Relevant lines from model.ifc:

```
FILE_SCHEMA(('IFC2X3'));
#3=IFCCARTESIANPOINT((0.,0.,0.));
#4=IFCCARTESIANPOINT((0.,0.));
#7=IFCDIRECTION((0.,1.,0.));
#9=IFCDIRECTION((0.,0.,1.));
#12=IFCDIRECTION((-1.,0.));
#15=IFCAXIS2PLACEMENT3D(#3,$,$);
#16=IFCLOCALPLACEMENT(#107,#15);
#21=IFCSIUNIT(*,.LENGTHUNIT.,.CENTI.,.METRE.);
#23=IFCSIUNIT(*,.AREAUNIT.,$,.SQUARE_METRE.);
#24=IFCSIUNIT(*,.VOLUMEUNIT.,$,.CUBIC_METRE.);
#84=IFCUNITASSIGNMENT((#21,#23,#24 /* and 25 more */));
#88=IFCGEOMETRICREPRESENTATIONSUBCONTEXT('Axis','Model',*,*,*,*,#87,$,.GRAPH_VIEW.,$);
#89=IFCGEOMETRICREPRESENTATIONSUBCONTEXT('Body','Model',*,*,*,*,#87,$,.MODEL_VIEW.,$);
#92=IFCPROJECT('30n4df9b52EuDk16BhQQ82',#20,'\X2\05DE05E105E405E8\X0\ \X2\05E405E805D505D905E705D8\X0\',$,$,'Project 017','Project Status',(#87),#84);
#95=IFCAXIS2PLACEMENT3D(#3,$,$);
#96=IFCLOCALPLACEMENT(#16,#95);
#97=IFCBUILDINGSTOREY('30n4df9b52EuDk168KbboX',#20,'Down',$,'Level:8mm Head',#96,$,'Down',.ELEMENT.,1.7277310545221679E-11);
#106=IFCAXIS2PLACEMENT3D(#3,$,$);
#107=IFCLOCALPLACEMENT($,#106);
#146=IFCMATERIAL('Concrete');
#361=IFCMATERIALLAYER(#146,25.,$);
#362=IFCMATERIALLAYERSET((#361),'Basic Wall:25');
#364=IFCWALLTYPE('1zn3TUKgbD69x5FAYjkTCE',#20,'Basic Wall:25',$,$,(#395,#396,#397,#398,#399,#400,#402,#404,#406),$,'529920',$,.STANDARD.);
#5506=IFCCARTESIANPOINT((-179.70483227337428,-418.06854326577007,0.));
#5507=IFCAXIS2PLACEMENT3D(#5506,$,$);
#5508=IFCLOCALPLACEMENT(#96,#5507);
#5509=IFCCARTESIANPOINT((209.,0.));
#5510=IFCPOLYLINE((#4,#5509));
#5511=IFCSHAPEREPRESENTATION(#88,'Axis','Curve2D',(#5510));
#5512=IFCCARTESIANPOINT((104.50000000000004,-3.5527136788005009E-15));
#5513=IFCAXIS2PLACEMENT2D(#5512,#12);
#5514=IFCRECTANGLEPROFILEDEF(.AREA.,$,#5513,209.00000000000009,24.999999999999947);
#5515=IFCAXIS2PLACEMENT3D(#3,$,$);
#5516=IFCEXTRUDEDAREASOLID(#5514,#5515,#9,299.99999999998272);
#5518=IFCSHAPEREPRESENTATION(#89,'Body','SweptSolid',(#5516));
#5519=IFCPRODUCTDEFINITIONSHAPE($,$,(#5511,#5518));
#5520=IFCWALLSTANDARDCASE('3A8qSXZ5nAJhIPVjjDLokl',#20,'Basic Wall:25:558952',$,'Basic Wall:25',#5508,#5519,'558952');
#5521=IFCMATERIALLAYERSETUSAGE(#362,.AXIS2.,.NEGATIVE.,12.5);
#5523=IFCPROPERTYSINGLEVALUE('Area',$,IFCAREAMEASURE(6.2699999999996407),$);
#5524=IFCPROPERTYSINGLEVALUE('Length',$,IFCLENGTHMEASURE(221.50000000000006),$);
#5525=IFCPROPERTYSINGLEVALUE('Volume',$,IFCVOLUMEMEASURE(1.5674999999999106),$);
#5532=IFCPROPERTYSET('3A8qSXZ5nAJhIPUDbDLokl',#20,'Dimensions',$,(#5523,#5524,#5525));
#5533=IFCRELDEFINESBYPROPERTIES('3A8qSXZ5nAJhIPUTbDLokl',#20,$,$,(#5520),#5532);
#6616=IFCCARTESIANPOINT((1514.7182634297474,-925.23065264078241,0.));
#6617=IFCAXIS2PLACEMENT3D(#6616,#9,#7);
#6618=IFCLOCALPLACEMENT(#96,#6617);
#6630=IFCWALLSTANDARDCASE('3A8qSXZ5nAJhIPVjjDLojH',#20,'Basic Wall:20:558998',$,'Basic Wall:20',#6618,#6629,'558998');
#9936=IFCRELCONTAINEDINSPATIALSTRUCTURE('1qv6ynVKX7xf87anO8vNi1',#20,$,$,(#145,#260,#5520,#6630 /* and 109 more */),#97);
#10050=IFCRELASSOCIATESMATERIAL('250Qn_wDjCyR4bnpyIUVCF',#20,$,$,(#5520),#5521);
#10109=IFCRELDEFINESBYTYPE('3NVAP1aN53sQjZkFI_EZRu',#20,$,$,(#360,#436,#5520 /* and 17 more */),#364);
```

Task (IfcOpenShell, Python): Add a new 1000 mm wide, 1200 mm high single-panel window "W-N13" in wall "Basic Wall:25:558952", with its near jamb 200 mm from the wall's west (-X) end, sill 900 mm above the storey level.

```python
import numpy as np
import ifcopenshell
import ifcopenshell.api.feature
import ifcopenshell.api.geometry
import ifcopenshell.api.pset
import ifcopenshell.api.root
import ifcopenshell.api.spatial
import ifcopenshell.api.type
import ifcopenshell.geom
import ifcopenshell.util.element
import ifcopenshell.util.placement
import ifcopenshell.util.representation
import ifcopenshell.util.shape
import ifcopenshell.util.unit

model = ifcopenshell.open("model.ifc")
unit_scale = ifcopenshell.util.unit.calculate_unit_scale(model)
area_scale = ifcopenshell.util.unit.calculate_unit_scale(model, "AREAUNIT")
volume_scale = ifcopenshell.util.unit.calculate_unit_scale(model, "VOLUMEUNIT")
settings = ifcopenshell.geom.settings()


def volume(element):
    """Net volume in cubic metres, openings subtracted."""
    shape = ifcopenshell.geom.create_shape(settings, element)
    return ifcopenshell.util.shape.get_volume(shape.geometry)


wall = model.by_guid("3A8qSXZ5nAJhIPVjjDLokl")
storey = ifcopenshell.util.element.get_container(wall, ifc_class="IfcBuildingStorey")
context = ifcopenshell.util.representation.get_context(model, "Model", "Body", "MODEL_VIEW")
before = volume(wall)

width, height, from_end, sill = 1, 1.2, 0.2, 0.9  # metres

# The wall runs along its own X axis, and the end named is its -X end.
wall_shape = ifcopenshell.geom.create_shape(settings, wall)
x, y, z = ifcopenshell.util.shape.get_vertices(wall_shape.geometry).T
start = x.min() + from_end
face, thickness = float(y.min()), float(y.max() - y.min())
wall_matrix = ifcopenshell.util.placement.get_local_placement(wall.ObjectPlacement)
level = ifcopenshell.util.placement.get_local_placement(storey.ObjectPlacement)[2, 3]


def in_wall(x, y):
    """Placement at x, y metres in the wall's axes, at sill height."""
    matrix = wall_matrix.copy()
    matrix[:, 3] = wall_matrix @ np.array([x / unit_scale, y / unit_scale, 0.0, 1.0])
    matrix[2, 3] = level + sill / unit_scale
    return matrix


# Opening: a box that overshoots both wall faces by 50 mm.
opening = ifcopenshell.api.root.create_entity(model, ifc_class="IfcOpeningElement")
box = ifcopenshell.api.geometry.add_wall_representation(
    model, context=context, length=width, height=height, thickness=thickness + 0.1
)
ifcopenshell.api.geometry.assign_representation(model, product=opening, representation=box)
ifcopenshell.api.geometry.edit_object_placement(model, product=opening, matrix=in_wall(start, face - 0.05), is_si=False)
ifcopenshell.api.feature.add_feature(model, feature=opening, element=wall)

window = ifcopenshell.api.root.create_entity(model, ifc_class="IfcWindow", name="W-N13")
window.OverallWidth, window.OverallHeight = width / unit_scale, height / unit_scale
body = ifcopenshell.api.geometry.add_window_representation(
    model,
    context=context,
    overall_width=window.OverallWidth,
    overall_height=window.OverallHeight,
    partition_type="SINGLE_PANEL",
)
ifcopenshell.api.geometry.assign_representation(model, product=window, representation=body)
ifcopenshell.api.spatial.assign_container(model, products=[window], relating_structure=storey)
fills = ifcopenshell.api.feature.add_filling(model, opening=opening, element=window)
fills.OwnerHistory = window.OwnerHistory  # required in IFC2X3

# IFC2X3 keeps the operation on the window style.
style = ifcopenshell.api.root.create_entity(model, ifc_class="IfcWindowStyle", name="W-N13")
style.OperationType, style.ConstructionType = "SINGLE_PANEL", "NOTDEFINED"
style.ParameterTakesPrecedence = style.Sizeable = False
ifcopenshell.api.type.assign_type(model, related_objects=[window], relating_type=style)

# Centre the window in the wall's thickness.
ifcopenshell.api.geometry.edit_object_placement(model, product=window, matrix=in_wall(start, face), is_si=False)
window_shape = ifcopenshell.geom.create_shape(settings, window)
depth = ifcopenshell.util.shape.get_vertices(window_shape.geometry)[:, 1]
offset = face + thickness / 2 - (depth.min() + depth.max()) / 2
ifcopenshell.api.geometry.edit_object_placement(model, product=window, matrix=in_wall(start, offset), is_si=False)

after = volume(wall)

# Update the wall's stored quantities.
pset = model.by_id(ifcopenshell.util.element.get_pset(wall, "Dimensions", should_inherit=False)["id"])
ifcopenshell.api.pset.edit_pset(model, pset=pset, properties={
    "Area": model.create_entity("IfcAreaMeasure", after / thickness / area_scale),
    "Volume": model.create_entity("IfcVolumeMeasure", after / volume_scale),
})

print(f"wall volume {before:.3f} -> {after:.3f} m3")

model.write("model_v2.ifc")
```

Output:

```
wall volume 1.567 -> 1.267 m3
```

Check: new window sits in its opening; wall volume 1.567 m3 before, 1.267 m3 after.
